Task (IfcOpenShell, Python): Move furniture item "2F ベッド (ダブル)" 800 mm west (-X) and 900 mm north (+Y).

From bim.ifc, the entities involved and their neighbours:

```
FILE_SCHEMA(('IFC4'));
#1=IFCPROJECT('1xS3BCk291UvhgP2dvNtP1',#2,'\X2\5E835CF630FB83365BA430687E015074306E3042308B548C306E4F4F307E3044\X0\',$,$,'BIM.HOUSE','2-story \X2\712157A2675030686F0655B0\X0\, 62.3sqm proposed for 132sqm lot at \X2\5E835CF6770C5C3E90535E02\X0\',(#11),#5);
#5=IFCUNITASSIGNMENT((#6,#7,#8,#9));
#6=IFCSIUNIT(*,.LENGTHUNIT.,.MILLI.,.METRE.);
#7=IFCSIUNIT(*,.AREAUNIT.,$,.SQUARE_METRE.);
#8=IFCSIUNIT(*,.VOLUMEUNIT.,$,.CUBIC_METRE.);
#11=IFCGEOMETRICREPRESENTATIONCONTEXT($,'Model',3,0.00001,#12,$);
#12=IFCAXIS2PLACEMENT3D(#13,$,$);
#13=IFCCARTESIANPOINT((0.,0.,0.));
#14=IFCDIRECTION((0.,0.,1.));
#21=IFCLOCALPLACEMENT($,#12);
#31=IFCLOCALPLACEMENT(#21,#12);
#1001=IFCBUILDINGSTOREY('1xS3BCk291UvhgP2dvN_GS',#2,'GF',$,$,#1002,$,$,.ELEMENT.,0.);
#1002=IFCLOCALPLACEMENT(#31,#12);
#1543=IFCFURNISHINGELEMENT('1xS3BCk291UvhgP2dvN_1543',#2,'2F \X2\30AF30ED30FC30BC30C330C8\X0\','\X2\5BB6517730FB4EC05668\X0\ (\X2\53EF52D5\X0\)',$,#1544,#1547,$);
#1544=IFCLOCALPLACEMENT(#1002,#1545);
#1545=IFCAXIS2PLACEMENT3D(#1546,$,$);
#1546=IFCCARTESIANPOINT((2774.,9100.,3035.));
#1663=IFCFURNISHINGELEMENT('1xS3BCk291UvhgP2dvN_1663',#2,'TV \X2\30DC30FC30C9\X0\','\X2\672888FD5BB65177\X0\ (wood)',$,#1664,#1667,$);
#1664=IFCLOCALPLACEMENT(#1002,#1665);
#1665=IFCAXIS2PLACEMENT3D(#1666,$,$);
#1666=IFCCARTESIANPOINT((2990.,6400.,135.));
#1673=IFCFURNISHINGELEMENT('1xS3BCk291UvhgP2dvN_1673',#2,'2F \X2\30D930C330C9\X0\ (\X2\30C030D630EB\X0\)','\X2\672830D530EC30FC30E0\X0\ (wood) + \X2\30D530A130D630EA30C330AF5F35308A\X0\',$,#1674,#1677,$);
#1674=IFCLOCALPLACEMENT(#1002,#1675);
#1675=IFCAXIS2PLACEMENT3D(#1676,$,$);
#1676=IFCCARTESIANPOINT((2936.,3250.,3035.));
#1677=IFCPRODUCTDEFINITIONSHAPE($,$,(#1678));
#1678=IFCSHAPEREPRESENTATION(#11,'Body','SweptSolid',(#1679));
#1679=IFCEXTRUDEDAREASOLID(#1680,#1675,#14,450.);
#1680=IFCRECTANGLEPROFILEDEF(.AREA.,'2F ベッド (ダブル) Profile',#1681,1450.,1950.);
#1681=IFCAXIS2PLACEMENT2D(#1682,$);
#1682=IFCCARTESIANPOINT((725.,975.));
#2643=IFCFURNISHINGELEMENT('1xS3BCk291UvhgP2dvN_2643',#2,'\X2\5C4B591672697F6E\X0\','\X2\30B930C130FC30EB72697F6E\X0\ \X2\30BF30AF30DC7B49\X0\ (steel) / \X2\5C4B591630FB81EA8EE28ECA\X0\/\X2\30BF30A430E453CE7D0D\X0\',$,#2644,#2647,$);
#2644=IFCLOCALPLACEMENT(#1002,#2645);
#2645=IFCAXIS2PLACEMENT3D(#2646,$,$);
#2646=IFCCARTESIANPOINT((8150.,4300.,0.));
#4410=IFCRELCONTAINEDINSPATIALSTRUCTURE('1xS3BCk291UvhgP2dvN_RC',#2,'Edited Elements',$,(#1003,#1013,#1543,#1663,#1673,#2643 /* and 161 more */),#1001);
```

```python
import ifcopenshell
import ifcopenshell.api.geometry
import ifcopenshell.util.placement
import ifcopenshell.util.unit

model = ifcopenshell.open("bim.ifc")
unit_scale = ifcopenshell.util.unit.calculate_unit_scale(model)

item = model.by_guid("1xS3BCk291UvhgP2dvN_1673")
matrix = ifcopenshell.util.placement.get_local_placement(item.ObjectPlacement)
matrix[0, 3] -= 0.8 / unit_scale
matrix[1, 3] += 0.9 / unit_scale
ifcopenshell.api.geometry.edit_object_placement(model, product=item, matrix=matrix, is_si=False)

print(ifcopenshell.util.placement.get_local_placement(item.ObjectPlacement).round(3) + 0.0)

model.write("bim_updated.ifc")
```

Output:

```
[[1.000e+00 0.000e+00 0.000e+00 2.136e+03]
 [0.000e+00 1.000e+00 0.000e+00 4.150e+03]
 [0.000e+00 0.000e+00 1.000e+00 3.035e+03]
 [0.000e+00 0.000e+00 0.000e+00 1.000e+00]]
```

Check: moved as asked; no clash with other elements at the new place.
